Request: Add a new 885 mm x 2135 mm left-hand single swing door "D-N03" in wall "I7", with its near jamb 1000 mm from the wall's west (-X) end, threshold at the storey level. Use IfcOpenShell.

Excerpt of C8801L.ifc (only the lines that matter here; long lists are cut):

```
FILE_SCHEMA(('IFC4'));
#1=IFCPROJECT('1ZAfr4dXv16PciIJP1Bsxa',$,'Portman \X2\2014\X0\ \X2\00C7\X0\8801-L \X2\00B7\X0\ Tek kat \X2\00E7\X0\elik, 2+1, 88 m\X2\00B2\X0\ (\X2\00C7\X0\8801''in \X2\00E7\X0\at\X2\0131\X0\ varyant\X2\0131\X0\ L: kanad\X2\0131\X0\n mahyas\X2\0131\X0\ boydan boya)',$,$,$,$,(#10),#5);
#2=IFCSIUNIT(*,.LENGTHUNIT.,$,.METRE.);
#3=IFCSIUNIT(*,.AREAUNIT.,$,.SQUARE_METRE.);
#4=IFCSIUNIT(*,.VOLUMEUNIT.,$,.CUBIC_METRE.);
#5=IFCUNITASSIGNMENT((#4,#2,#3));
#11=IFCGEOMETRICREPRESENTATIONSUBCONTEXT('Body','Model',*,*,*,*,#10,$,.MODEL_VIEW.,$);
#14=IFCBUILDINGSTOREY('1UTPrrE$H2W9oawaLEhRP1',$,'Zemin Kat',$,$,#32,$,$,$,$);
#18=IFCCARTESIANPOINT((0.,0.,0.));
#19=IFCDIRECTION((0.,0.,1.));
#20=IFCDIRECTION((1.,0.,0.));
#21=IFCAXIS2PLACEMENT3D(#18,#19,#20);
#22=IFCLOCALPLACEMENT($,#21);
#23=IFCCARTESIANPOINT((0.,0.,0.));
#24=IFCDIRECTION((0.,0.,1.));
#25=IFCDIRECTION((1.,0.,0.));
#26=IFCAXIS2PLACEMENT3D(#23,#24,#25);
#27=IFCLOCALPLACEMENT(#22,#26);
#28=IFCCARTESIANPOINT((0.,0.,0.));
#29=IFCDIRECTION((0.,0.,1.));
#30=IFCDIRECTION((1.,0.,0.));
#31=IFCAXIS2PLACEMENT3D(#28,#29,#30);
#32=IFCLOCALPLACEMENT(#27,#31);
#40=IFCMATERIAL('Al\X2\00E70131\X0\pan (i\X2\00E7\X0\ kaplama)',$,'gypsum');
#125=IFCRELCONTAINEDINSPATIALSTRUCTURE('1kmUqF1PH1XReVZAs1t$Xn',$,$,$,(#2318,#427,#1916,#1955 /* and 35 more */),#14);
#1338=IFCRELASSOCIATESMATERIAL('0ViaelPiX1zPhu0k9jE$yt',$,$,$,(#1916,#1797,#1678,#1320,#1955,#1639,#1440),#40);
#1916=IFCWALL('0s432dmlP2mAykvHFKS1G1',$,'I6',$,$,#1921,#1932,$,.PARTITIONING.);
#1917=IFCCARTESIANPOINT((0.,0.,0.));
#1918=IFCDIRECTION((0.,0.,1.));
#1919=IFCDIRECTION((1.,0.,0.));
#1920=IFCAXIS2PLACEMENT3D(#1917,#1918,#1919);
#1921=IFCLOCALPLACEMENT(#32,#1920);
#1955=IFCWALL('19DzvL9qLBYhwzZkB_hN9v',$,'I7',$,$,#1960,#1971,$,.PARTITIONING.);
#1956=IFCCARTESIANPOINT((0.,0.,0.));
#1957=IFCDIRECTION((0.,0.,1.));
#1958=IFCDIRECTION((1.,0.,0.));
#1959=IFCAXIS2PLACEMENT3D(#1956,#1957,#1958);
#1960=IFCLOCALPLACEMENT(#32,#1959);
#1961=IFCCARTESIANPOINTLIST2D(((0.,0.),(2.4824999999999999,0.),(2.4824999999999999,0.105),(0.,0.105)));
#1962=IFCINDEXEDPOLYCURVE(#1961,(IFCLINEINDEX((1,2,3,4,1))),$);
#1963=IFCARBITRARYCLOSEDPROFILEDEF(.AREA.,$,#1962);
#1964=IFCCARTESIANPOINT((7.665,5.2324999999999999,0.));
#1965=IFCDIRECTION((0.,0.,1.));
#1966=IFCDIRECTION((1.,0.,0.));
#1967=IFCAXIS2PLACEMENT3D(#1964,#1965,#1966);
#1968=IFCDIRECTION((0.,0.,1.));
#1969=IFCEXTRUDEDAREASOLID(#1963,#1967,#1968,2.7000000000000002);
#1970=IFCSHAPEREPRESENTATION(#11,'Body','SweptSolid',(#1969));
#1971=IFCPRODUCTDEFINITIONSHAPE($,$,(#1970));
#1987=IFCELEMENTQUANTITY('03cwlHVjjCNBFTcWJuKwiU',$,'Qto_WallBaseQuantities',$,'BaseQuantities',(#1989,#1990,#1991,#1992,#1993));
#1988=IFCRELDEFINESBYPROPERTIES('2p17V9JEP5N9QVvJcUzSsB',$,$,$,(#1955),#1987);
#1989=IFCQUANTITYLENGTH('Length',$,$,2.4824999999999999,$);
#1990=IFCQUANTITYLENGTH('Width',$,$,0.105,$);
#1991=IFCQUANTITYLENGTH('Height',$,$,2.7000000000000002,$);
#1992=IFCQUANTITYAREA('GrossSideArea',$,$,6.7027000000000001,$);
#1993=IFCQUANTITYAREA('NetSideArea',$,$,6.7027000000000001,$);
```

```python
import numpy as np
import ifcopenshell
import ifcopenshell.api.feature
import ifcopenshell.api.geometry
import ifcopenshell.api.pset
import ifcopenshell.api.root
import ifcopenshell.api.spatial
import ifcopenshell.geom
import ifcopenshell.util.element
import ifcopenshell.util.placement
import ifcopenshell.util.representation
import ifcopenshell.util.shape
import ifcopenshell.util.unit

model = ifcopenshell.open("C8801L.ifc")
unit_scale = ifcopenshell.util.unit.calculate_unit_scale(model)
area_scale = ifcopenshell.util.unit.calculate_unit_scale(model, "AREAUNIT")
settings = ifcopenshell.geom.settings()


def volume(element):
    """Net volume in cubic metres, openings subtracted."""
    shape = ifcopenshell.geom.create_shape(settings, element)
    return ifcopenshell.util.shape.get_volume(shape.geometry)


wall = model.by_guid("19DzvL9qLBYhwzZkB_hN9v")
storey = ifcopenshell.util.element.get_container(wall, ifc_class="IfcBuildingStorey")
context = ifcopenshell.util.representation.get_context(model, "Model", "Body", "MODEL_VIEW")
before = volume(wall)

width, height, from_end, sill = 0.885, 2.135, 1, 0.0  # metres

# The wall runs along its own X axis, and the end named is its -X end.
wall_shape = ifcopenshell.geom.create_shape(settings, wall)
x, y, z = ifcopenshell.util.shape.get_vertices(wall_shape.geometry).T
start = x.min() + from_end
face, thickness = float(y.min()), float(y.max() - y.min())
wall_matrix = ifcopenshell.util.placement.get_local_placement(wall.ObjectPlacement)
level = ifcopenshell.util.placement.get_local_placement(storey.ObjectPlacement)[2, 3]


def in_wall(x, y):
    """Placement at x, y metres in the wall's axes, at sill height."""
    matrix = wall_matrix.copy()
    matrix[:, 3] = wall_matrix @ np.array([x / unit_scale, y / unit_scale, 0.0, 1.0])
    matrix[2, 3] = level + sill / unit_scale
    return matrix


# Opening: a box that overshoots both wall faces by 50 mm.
opening = ifcopenshell.api.root.create_entity(model, ifc_class="IfcOpeningElement", predefined_type="OPENING")
box = ifcopenshell.api.geometry.add_wall_representation(
    model, context=context, length=width, height=height, thickness=thickness + 0.1
)
ifcopenshell.api.geometry.assign_representation(model, product=opening, representation=box)
ifcopenshell.api.geometry.edit_object_placement(model, product=opening, matrix=in_wall(start, face - 0.05), is_si=False)
ifcopenshell.api.feature.add_feature(model, feature=opening, element=wall)

door = ifcopenshell.api.root.create_entity(model, ifc_class="IfcDoor", name="D-N03", predefined_type="DOOR")
door.OverallWidth, door.OverallHeight = width / unit_scale, height / unit_scale
door.OperationType = "SINGLE_SWING_LEFT"
body = ifcopenshell.api.geometry.add_door_representation(
    model,
    context=context,
    overall_width=door.OverallWidth,
    overall_height=door.OverallHeight,
    operation_type="SINGLE_SWING_LEFT",
    lining_properties={"LiningDepth": thickness / unit_scale, "ThresholdDepth": thickness / unit_scale},
)
ifcopenshell.api.geometry.assign_representation(model, product=door, representation=body)
ifcopenshell.api.spatial.assign_container(model, products=[door], relating_structure=storey)
ifcopenshell.api.feature.add_filling(model, opening=opening, element=door)

# The lining spans the wall, so the door starts at the wall face.
ifcopenshell.api.geometry.edit_object_placement(model, product=door, matrix=in_wall(start, face), is_si=False)

after = volume(wall)

# Update the wall's stored quantities.
qto = model.by_id(ifcopenshell.util.element.get_pset(wall, "Qto_WallBaseQuantities", should_inherit=False)["id"])
ifcopenshell.api.pset.edit_qto(model, qto=qto, properties={"NetSideArea": after / thickness / area_scale})

print(f"wall volume {before:.3f} -> {after:.3f} m3")

model.write("C8801L_v2.ifc")
```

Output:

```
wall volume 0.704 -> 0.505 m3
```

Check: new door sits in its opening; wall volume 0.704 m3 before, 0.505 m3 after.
